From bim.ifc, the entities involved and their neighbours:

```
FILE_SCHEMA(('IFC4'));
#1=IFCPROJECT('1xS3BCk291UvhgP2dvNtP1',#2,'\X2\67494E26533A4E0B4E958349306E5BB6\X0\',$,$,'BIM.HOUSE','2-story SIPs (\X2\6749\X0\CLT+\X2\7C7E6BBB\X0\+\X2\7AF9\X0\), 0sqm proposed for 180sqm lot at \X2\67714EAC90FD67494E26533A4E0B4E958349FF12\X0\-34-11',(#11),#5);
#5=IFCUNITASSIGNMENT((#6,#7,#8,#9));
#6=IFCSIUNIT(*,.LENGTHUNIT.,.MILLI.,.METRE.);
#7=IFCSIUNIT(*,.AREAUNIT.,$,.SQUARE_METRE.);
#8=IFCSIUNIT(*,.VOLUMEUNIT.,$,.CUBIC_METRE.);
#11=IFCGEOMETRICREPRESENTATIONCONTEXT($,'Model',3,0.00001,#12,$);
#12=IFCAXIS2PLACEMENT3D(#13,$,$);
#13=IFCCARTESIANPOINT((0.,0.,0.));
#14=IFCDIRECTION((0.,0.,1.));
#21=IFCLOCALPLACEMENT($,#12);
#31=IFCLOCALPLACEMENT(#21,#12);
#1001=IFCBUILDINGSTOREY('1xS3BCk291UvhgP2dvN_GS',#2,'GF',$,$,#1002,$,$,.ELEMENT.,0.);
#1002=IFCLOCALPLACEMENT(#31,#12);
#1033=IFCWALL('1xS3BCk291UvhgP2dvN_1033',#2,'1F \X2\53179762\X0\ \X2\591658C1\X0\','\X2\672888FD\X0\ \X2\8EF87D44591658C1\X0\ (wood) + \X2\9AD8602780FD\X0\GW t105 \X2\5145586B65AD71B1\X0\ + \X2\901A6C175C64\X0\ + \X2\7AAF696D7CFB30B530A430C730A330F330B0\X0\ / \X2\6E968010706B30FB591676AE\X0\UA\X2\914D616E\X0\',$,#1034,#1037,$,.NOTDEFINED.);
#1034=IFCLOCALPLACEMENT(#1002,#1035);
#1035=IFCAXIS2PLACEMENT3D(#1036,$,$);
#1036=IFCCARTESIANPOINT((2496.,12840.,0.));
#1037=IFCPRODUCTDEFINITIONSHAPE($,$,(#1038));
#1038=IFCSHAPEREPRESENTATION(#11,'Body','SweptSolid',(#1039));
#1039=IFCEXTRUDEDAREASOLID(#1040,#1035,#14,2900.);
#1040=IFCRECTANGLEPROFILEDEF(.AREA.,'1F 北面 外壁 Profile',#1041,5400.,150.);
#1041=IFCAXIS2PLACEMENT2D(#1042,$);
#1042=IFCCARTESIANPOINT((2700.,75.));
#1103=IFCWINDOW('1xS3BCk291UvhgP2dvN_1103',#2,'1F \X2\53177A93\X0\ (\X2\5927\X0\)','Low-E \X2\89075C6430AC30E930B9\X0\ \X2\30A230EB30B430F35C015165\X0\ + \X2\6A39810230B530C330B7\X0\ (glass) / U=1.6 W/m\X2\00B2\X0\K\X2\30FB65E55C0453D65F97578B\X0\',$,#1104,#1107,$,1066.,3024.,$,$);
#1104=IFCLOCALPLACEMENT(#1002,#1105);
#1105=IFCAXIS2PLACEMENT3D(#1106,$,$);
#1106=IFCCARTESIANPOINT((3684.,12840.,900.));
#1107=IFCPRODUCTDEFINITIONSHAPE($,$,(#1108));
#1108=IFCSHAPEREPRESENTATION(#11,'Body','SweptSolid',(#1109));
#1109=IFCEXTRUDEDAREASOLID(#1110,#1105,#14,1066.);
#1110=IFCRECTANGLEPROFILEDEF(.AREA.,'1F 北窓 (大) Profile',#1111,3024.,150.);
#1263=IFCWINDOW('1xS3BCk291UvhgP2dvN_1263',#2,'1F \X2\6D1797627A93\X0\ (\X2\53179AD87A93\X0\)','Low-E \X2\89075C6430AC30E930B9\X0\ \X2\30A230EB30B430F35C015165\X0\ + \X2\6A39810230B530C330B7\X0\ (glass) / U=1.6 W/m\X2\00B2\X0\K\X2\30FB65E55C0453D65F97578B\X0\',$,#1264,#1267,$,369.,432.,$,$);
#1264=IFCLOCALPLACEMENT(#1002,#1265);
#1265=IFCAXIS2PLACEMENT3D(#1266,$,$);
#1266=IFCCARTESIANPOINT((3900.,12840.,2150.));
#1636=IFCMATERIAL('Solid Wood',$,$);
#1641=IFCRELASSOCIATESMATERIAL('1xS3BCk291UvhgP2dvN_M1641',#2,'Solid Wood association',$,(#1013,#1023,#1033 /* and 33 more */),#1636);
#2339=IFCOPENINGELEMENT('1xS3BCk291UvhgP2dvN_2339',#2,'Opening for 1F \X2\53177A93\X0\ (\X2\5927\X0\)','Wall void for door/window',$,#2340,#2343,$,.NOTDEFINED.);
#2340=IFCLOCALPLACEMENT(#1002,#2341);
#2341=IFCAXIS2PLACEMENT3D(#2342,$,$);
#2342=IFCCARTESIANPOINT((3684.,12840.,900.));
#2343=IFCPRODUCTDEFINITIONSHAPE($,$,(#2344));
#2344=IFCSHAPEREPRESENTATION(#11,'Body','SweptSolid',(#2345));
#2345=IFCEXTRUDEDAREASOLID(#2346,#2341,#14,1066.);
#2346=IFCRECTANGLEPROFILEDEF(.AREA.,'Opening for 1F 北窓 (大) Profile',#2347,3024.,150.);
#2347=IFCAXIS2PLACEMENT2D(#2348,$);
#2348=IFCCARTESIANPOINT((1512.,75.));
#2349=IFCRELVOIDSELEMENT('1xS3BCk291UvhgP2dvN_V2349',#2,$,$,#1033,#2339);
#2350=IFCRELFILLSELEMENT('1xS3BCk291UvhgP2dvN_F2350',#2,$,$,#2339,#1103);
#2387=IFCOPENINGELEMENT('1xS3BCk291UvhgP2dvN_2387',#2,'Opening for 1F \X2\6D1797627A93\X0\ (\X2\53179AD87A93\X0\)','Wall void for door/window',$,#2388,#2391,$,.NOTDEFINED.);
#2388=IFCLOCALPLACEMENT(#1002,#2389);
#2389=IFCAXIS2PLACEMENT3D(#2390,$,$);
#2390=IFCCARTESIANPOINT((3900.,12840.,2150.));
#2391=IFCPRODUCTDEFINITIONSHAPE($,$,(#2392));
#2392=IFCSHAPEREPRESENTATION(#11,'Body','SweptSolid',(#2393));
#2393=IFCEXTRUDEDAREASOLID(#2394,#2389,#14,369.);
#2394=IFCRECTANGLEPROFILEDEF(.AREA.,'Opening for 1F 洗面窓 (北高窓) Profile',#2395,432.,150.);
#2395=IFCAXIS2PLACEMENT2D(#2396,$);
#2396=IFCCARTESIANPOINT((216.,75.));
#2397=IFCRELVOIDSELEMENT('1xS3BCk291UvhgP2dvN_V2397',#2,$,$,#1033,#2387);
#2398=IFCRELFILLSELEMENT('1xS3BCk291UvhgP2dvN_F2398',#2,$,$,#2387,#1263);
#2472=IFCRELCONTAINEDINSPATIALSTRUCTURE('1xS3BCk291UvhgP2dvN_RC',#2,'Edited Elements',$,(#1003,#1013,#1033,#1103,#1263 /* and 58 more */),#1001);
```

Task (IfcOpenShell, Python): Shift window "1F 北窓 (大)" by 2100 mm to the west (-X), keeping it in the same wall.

```python
import ifcopenshell
import ifcopenshell.api.geometry
import ifcopenshell.util.placement

model = ifcopenshell.open("bim.ifc")

window = model.by_guid("1xS3BCk291UvhgP2dvN_1103")
opening = window.FillsVoids[0].RelatingOpeningElement
wall = opening.VoidsElements[0].RelatingBuildingElement

wall_matrix = ifcopenshell.util.placement.get_local_placement(wall.ObjectPlacement)
shift = wall_matrix[:3, 0] * -2100.0
before = ifcopenshell.util.placement.get_local_placement(window.ObjectPlacement)[:3, 3].copy()

# The window is not placed relative to its opening, so move both.
for product in (opening, window):
    matrix = ifcopenshell.util.placement.get_local_placement(product.ObjectPlacement)
    matrix[:3, 3] += shift
    ifcopenshell.api.geometry.edit_object_placement(model, product=product, matrix=matrix, is_si=False)

after = ifcopenshell.util.placement.get_local_placement(window.ObjectPlacement)[:3, 3]
print("window moved by", (after - before).round(3) + 0.0)

model.write("bim-out.ifc")
```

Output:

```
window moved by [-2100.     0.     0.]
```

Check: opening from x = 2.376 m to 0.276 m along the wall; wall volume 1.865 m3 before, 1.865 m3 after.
